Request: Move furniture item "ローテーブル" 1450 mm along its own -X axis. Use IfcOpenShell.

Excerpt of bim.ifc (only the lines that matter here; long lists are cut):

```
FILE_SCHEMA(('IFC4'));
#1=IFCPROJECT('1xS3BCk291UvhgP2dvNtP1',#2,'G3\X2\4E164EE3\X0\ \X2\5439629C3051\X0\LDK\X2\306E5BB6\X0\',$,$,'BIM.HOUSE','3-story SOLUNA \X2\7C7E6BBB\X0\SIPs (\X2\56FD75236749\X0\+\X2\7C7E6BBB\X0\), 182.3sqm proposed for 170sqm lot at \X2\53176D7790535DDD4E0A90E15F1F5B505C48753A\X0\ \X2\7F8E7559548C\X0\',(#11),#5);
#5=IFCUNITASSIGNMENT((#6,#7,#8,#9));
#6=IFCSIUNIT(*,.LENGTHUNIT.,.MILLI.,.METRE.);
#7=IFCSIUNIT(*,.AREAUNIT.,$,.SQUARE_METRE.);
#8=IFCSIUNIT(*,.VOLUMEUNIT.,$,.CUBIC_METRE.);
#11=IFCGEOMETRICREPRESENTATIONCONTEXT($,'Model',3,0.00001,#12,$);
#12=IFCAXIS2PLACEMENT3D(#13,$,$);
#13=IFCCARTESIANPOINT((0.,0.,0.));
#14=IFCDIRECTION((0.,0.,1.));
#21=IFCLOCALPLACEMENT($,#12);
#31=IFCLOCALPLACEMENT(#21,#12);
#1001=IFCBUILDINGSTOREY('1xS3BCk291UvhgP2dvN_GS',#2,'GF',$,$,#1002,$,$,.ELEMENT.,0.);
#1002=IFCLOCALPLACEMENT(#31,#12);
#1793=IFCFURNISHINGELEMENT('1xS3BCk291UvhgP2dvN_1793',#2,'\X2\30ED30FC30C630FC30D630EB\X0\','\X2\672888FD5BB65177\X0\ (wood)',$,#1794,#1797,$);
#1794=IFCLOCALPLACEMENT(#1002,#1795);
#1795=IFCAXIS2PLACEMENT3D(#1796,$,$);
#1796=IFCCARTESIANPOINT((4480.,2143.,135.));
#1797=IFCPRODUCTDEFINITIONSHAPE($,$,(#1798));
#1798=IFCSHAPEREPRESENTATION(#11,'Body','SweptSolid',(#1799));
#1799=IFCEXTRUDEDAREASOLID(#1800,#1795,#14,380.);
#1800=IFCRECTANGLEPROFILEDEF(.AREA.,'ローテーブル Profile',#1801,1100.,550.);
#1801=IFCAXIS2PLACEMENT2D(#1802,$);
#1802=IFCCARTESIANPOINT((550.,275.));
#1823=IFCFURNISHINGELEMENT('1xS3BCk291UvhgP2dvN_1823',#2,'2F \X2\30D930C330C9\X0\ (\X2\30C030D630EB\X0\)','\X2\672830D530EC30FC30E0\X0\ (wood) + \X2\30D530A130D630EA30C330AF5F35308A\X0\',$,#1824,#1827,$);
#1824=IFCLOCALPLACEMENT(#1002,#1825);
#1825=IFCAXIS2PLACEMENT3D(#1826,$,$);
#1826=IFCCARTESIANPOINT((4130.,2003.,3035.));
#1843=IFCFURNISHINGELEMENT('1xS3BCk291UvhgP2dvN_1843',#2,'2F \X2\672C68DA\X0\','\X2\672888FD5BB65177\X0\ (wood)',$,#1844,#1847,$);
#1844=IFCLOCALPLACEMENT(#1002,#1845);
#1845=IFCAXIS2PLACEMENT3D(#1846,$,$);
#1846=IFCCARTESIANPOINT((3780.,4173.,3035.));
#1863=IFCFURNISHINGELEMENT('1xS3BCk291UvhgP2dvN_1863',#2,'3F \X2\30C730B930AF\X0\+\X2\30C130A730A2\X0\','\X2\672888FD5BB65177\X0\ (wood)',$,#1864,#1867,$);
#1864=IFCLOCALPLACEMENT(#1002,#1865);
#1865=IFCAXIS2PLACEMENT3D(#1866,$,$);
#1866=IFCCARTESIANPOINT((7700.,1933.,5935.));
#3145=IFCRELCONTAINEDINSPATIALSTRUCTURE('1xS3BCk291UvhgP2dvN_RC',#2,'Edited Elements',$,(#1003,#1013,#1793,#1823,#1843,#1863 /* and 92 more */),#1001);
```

```python
import ifcopenshell
import ifcopenshell.api.geometry
import ifcopenshell.util.placement
import ifcopenshell.util.unit

model = ifcopenshell.open("bim.ifc")
unit_scale = ifcopenshell.util.unit.calculate_unit_scale(model)

item = model.by_guid("1xS3BCk291UvhgP2dvN_1793")
matrix = ifcopenshell.util.placement.get_local_placement(item.ObjectPlacement)
matrix[:3, 3] -= matrix[:3, 0] * 1.45 / unit_scale
ifcopenshell.api.geometry.edit_object_placement(model, product=item, matrix=matrix, is_si=False)

print(ifcopenshell.util.placement.get_local_placement(item.ObjectPlacement).round(3) + 0.0)

model.write("bim_v2.ifc")
```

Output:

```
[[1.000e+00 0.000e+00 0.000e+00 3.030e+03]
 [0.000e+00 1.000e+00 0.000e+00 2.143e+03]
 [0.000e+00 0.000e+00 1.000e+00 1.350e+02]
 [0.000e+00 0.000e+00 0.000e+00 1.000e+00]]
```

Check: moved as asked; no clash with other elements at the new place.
